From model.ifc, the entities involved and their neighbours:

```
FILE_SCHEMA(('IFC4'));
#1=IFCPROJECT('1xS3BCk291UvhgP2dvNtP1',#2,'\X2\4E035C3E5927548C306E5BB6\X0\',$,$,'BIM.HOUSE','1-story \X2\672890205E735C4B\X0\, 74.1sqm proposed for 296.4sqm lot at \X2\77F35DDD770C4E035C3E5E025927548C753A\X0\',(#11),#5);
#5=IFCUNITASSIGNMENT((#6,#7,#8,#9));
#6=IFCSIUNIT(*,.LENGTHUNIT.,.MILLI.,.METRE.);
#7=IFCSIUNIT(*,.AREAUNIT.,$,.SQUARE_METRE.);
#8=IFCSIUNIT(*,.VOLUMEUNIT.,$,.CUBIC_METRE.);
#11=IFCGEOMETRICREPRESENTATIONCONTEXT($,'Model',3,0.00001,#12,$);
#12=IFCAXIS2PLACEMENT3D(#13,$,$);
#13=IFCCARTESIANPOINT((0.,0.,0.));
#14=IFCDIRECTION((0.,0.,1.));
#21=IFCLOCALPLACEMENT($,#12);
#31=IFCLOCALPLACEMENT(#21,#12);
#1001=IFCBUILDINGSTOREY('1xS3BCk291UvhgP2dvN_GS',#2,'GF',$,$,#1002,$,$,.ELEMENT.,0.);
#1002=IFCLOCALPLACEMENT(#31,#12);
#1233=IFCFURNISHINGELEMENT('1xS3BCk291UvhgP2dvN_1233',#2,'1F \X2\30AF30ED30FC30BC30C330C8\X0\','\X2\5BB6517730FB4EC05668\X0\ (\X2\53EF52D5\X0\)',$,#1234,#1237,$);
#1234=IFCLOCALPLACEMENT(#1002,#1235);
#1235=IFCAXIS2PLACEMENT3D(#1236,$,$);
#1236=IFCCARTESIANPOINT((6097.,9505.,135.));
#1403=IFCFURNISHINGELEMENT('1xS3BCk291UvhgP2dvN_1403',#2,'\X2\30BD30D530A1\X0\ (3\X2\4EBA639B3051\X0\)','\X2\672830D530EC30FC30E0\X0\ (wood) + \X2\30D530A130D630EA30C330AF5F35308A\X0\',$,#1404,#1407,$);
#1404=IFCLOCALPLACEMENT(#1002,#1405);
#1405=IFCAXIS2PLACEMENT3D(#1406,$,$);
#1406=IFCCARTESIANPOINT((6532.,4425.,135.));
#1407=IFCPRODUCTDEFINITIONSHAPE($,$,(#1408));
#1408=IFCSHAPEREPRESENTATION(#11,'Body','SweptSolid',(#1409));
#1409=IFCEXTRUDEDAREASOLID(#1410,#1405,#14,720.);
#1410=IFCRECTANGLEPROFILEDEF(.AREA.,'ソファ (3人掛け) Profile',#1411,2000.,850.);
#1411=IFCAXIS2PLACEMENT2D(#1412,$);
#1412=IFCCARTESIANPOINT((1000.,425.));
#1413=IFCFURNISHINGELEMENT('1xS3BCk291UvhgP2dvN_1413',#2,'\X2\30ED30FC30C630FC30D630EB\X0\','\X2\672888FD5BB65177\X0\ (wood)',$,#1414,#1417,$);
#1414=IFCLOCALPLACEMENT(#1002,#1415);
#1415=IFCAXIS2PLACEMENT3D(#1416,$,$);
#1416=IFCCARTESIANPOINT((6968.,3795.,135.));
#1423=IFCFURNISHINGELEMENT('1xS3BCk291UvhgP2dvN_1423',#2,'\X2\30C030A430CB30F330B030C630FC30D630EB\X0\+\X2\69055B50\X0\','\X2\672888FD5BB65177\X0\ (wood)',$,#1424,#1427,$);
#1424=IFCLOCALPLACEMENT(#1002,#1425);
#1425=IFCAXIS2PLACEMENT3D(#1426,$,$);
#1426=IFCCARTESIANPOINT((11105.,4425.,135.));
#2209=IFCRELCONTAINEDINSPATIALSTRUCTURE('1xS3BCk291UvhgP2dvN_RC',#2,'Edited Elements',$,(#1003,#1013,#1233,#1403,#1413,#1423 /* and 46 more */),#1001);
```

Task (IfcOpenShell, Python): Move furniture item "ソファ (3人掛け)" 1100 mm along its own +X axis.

```python
import ifcopenshell
import ifcopenshell.api.geometry
import ifcopenshell.util.placement

model = ifcopenshell.open("model.ifc")

item = model.by_guid("1xS3BCk291UvhgP2dvN_1403")
matrix = ifcopenshell.util.placement.get_local_placement(item.ObjectPlacement)
matrix[:3, 3] += matrix[:3, 0] * 1100.0
ifcopenshell.api.geometry.edit_object_placement(model, product=item, matrix=matrix, is_si=False)

print(ifcopenshell.util.placement.get_local_placement(item.ObjectPlacement).round(3) + 0.0)

model.write("model_edited.ifc")
```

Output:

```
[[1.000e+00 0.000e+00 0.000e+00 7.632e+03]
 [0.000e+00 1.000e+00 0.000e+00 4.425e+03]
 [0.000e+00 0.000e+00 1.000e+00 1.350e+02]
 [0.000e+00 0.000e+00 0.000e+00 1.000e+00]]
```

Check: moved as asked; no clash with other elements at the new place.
